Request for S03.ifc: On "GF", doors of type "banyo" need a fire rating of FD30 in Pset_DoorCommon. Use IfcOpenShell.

First a look at what the model holds.

```python
import ifcopenshell
import ifcopenshell.util.element

model = ifcopenshell.open("S03.ifc")
print(model.schema)
storey = next(s for s in model.by_type("IfcBuildingStorey") if s.Name == "GF")
doors = [e for e in ifcopenshell.util.element.get_decomposition(storey) if e.is_a("IfcDoor")]
seen = {}
for e in doors:
    element_type = ifcopenshell.util.element.get_type(e)
    key = (element_type.Name if element_type != e and element_type else None, ifcopenshell.util.element.get_pset(e, "Pset_DoorCommon", "FireRating"))
    seen[key] = seen.get(key, 0) + 1
for (name, value), count in sorted(seen.items(), key=str):
    print(count, "x", name, "|", value)
```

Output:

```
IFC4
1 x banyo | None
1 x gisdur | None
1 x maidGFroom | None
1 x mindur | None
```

```python
import ifcopenshell
import ifcopenshell.api.pset
import ifcopenshell.util.element

model = ifcopenshell.open("S03.ifc")

storey = next(s for s in model.by_type("IfcBuildingStorey") if s.Name == "GF")
doors = [e for e in ifcopenshell.util.element.get_decomposition(storey) if e.is_a("IfcDoor")]

count = 0
for e in doors:
    element_type = ifcopenshell.util.element.get_type(e)
    if element_type in (None, e) or element_type.Name != "banyo":
        continue
    # add_pset returns the element's existing set when there is one.
    pset = ifcopenshell.api.pset.add_pset(model, product=e, name="Pset_DoorCommon")
    ifcopenshell.api.pset.edit_pset(model, pset=pset, properties={"FireRating": "FD30"})
    count += 1

print(count, "doors updated")

model.write("S03-out.ifc")
```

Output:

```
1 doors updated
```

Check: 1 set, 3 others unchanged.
